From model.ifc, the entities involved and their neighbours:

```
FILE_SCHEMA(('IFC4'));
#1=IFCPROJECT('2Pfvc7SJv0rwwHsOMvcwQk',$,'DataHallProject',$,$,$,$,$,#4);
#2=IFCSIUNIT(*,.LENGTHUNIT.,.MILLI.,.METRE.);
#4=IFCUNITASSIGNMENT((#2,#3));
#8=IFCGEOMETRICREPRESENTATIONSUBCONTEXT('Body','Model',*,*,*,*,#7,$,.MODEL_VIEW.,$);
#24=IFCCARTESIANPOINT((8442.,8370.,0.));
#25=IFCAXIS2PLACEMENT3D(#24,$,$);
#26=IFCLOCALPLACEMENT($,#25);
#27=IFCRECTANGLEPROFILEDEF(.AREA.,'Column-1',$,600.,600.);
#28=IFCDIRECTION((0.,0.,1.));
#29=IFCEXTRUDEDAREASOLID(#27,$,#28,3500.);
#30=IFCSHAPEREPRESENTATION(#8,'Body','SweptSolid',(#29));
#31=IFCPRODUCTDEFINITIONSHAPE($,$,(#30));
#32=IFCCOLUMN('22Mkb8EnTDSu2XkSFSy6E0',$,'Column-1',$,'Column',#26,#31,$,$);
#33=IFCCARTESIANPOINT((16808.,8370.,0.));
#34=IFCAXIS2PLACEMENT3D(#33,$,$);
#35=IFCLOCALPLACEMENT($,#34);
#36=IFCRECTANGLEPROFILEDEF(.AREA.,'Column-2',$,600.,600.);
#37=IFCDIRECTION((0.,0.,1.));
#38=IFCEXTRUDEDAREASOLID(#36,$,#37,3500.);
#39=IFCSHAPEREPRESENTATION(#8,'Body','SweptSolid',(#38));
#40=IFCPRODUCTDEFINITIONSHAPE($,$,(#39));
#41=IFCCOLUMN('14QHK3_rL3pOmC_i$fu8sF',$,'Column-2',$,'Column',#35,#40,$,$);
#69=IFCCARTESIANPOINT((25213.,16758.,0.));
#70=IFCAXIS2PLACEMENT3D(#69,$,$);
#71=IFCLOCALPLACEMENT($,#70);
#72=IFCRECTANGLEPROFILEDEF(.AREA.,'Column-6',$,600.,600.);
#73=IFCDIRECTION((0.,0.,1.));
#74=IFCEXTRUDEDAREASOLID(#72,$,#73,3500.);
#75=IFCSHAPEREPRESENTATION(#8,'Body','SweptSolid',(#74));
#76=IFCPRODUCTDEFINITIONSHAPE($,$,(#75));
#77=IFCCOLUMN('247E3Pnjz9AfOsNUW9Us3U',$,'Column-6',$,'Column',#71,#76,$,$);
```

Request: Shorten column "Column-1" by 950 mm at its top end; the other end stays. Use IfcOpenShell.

```python
import ifcopenshell
import ifcopenshell.util.representation
import ifcopenshell.util.unit

model = ifcopenshell.open("model.ifc")
unit_scale = ifcopenshell.util.unit.calculate_unit_scale(model)

member = model.by_guid("22Mkb8EnTDSu2XkSFSy6E0")
change = -0.95 / unit_scale

# The extrusion runs towards the end named, so only its depth changes.
body = ifcopenshell.util.representation.get_representation(member, "Model", "Body")
solid = body.Items[0]
old_length = solid.Depth
solid.Depth += change

print(f"length {old_length:g} -> {solid.Depth:g}")

model.write("model-out.ifc")
```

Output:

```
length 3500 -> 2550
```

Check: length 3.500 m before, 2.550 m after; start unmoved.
